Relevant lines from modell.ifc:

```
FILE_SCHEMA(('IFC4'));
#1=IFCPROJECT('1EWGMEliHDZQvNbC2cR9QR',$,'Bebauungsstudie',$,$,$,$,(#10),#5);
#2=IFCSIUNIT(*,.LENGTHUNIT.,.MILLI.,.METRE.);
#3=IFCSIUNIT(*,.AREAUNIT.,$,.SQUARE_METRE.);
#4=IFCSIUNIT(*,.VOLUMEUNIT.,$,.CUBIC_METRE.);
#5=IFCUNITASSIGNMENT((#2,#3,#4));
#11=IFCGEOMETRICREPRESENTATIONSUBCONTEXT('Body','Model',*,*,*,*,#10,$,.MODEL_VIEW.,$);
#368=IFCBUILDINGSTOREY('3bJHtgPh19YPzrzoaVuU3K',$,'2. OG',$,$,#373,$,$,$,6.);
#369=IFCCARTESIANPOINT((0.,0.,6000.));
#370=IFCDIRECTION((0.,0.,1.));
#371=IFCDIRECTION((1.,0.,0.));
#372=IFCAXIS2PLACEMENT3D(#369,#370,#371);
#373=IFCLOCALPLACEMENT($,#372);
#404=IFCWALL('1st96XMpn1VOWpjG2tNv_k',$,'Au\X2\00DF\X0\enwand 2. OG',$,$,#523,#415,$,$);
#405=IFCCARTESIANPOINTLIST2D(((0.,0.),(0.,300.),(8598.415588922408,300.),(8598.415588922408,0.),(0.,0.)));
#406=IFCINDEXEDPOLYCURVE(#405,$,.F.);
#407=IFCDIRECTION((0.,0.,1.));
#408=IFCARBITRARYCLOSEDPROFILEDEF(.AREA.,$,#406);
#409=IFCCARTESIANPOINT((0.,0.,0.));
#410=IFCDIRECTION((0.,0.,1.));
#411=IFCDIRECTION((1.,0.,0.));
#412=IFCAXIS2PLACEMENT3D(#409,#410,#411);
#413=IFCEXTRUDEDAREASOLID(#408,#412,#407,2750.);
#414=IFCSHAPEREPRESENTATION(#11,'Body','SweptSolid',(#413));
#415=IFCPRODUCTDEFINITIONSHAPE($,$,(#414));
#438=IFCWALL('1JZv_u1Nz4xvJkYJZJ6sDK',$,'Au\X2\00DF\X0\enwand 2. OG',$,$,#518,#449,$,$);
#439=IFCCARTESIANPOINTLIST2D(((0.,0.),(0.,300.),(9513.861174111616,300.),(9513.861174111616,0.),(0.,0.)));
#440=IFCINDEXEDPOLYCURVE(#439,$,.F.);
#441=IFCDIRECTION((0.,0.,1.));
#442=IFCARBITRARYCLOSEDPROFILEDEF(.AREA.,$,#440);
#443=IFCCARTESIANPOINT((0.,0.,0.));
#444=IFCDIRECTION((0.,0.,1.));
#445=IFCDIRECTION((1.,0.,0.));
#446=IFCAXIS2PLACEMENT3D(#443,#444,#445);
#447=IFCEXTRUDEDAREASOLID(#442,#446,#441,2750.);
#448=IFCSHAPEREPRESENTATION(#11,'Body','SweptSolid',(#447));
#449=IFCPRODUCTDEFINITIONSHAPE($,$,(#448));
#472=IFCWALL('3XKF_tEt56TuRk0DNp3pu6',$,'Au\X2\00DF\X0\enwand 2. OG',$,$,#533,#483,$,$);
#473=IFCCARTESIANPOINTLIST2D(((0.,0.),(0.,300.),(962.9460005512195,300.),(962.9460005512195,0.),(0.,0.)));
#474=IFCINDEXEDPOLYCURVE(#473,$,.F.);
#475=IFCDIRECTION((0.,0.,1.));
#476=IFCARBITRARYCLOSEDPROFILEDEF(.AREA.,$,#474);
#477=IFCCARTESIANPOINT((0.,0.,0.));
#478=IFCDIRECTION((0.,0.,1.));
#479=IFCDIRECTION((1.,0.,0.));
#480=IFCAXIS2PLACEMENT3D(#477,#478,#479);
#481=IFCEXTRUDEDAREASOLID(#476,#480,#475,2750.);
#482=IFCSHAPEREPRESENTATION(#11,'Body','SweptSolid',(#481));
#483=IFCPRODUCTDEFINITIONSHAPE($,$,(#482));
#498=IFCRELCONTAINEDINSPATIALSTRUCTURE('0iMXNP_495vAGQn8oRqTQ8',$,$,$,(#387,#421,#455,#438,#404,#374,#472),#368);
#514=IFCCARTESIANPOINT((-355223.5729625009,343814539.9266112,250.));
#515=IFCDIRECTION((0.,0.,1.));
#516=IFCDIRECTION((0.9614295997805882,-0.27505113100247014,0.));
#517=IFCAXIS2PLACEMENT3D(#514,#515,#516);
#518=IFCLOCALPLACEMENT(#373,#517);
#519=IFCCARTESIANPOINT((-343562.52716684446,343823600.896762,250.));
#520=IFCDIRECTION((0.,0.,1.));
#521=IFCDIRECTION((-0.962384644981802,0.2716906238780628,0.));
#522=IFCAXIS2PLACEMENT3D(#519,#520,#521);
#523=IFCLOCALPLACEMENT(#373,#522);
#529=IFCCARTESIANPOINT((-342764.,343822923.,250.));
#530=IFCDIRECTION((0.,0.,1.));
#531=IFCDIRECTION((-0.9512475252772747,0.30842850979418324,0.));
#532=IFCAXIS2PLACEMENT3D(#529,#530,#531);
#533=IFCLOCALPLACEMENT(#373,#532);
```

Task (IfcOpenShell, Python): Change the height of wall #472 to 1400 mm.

```python
import ifcopenshell
import ifcopenshell.geom
import ifcopenshell.util.representation
import ifcopenshell.util.shape
import ifcopenshell.util.unit

model = ifcopenshell.open("modell.ifc")
unit_scale = ifcopenshell.util.unit.calculate_unit_scale(model)
settings = ifcopenshell.geom.settings()


def volume(element):
    """Net volume in cubic metres, openings subtracted."""
    shape = ifcopenshell.geom.create_shape(settings, element)
    return ifcopenshell.util.shape.get_volume(shape.geometry)


wall = model.by_id(472)
before = volume(wall)

body = ifcopenshell.util.representation.get_representation(wall, "Model", "Body")
solid = body.Items[0]
old_height = solid.Depth
solid.Depth = 1.4 / unit_scale
after = volume(wall)

print(f"height {old_height:g} -> {solid.Depth:g}, volume {before:.3f} -> {after:.3f} m3")

model.write("modell_v2.ifc")
```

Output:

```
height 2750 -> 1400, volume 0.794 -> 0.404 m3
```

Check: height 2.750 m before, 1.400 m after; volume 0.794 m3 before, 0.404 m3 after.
